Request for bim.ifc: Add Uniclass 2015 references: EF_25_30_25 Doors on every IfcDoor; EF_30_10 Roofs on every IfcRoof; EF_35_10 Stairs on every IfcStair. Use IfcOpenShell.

First a look at what the model holds.

```python
import ifcopenshell

model = ifcopenshell.open("bim.ifc")
print(model.schema)
print("classifications:", [c.Name for c in model.by_type("IfcClassification")])
for ifc_class in ("IfcDoor", "IfcRoof", "IfcStair", "IfcWall", "IfcWindow"):
    print(ifc_class, len(model.by_type(ifc_class)))
```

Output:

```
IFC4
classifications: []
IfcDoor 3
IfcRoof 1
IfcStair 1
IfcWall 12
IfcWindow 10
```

```python
import ifcopenshell
import ifcopenshell.api.classification

model = ifcopenshell.open("bim.ifc")

system = ifcopenshell.api.classification.add_classification(model, classification="Uniclass 2015")

codes = {
    "IfcDoor": ("EF_25_30_25", "Doors"),
    "IfcRoof": ("EF_30_10", "Roofs"),
    "IfcStair": ("EF_35_10", "Stairs"),
}
for ifc_class, (code, name) in codes.items():
    products = model.by_type(ifc_class)
    ifcopenshell.api.classification.add_reference(
        model, products=products, classification=system, identification=code, name=name
    )
    print(code, len(products))

model.write("bim_rev.ifc")
```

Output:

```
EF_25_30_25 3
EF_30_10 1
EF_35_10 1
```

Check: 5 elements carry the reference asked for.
